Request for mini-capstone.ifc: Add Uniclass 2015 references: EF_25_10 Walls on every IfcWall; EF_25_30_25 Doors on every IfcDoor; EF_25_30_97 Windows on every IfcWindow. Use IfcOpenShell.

First a look at what the model holds.

```python
import ifcopenshell

model = ifcopenshell.open("mini-capstone.ifc")
print(model.schema)
print("classifications:", [c.Name for c in model.by_type("IfcClassification")])
for ifc_class in ("IfcDoor", "IfcRoof", "IfcStair", "IfcWall", "IfcWindow"):
    print(ifc_class, len(model.by_type(ifc_class)))
```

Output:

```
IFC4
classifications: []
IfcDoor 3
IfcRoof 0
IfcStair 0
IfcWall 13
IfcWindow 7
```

```python
import ifcopenshell
import ifcopenshell.api.classification

model = ifcopenshell.open("mini-capstone.ifc")

system = ifcopenshell.api.classification.add_classification(model, classification="Uniclass 2015")

codes = {
    "IfcWall": ("EF_25_10", "Walls"),
    "IfcDoor": ("EF_25_30_25", "Doors"),
    "IfcWindow": ("EF_25_30_97", "Windows"),
}
for ifc_class, (code, name) in codes.items():
    products = model.by_type(ifc_class)
    ifcopenshell.api.classification.add_reference(
        model, products=products, classification=system, identification=code, name=name
    )
    print(code, len(products))

model.write("mini-capstone_v2.ifc")
```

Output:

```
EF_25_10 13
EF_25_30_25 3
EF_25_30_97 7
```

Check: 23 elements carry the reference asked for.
